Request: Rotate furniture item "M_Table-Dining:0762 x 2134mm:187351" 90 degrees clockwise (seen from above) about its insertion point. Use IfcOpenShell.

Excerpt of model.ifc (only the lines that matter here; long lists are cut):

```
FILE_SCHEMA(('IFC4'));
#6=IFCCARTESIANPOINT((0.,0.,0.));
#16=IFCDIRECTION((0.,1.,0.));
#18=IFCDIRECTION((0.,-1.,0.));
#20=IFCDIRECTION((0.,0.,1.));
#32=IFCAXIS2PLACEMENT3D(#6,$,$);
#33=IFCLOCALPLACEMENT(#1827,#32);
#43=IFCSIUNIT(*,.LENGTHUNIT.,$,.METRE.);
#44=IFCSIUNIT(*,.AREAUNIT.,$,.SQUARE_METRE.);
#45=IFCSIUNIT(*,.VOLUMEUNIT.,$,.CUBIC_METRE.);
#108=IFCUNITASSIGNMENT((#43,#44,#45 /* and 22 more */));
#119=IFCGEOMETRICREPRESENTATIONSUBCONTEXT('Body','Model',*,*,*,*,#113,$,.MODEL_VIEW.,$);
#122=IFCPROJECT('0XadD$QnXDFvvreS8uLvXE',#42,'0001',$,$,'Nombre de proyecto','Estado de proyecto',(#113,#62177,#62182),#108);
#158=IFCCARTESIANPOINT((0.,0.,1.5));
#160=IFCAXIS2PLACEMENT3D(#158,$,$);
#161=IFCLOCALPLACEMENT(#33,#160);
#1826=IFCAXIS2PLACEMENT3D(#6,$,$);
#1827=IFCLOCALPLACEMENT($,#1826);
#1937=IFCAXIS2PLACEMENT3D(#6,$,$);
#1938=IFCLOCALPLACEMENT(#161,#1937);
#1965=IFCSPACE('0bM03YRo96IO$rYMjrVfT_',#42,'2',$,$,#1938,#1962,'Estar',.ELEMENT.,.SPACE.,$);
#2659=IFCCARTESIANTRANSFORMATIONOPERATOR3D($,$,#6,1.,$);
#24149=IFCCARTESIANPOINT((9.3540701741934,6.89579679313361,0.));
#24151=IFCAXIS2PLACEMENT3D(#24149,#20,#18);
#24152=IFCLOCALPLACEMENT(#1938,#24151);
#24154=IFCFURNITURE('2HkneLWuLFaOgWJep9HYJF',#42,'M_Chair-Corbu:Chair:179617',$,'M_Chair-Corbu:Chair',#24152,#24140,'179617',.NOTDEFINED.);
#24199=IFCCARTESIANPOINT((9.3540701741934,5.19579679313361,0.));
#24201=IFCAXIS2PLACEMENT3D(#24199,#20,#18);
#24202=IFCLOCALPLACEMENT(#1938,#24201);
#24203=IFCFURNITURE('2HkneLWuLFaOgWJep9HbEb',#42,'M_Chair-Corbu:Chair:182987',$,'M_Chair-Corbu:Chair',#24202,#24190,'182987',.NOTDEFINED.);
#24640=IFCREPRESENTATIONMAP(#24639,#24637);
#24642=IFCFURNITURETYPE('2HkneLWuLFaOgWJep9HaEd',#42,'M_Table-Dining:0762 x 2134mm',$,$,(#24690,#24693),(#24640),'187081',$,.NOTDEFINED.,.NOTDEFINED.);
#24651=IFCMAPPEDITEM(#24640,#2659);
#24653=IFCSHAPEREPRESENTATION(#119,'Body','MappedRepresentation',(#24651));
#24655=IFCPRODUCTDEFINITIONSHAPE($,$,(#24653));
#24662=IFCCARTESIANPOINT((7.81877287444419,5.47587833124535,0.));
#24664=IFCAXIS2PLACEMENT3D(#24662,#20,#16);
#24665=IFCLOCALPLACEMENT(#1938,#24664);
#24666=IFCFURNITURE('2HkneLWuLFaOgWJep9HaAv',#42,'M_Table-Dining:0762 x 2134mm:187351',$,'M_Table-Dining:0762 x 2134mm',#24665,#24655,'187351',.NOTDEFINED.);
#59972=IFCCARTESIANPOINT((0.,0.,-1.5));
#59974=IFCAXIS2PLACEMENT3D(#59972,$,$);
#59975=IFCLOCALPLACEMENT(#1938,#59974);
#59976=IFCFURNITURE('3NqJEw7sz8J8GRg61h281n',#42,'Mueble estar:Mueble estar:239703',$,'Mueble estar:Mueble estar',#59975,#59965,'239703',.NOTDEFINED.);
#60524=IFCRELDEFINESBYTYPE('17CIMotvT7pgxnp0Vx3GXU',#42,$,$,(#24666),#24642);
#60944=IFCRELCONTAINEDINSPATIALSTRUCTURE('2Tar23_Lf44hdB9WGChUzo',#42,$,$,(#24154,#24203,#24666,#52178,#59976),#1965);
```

```python
import ifcopenshell
import ifcopenshell.api.geometry
import ifcopenshell.util.placement

model = ifcopenshell.open("model.ifc")

item = model.by_guid("2HkneLWuLFaOgWJep9HaAv")
matrix = ifcopenshell.util.placement.get_local_placement(item.ObjectPlacement)
matrix = matrix @ ifcopenshell.util.placement.rotation(-90, "Z")
ifcopenshell.api.geometry.edit_object_placement(model, product=item, matrix=matrix, is_si=False)

print(ifcopenshell.util.placement.get_local_placement(item.ObjectPlacement).round(3) + 0.0)

model.write("model-out.ifc")
```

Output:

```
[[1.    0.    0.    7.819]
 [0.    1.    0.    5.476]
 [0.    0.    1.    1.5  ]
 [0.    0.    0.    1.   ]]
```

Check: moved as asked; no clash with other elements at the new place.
